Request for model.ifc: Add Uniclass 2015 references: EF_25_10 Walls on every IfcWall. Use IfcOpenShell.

First a look at what the model holds.

```python
import ifcopenshell

model = ifcopenshell.open("model.ifc")
print(model.schema)
print("classifications:", [c.Name for c in model.by_type("IfcClassification")])
for ifc_class in ("IfcDoor", "IfcRoof", "IfcStair", "IfcWall", "IfcWindow"):
    print(ifc_class, len(model.by_type(ifc_class)))
```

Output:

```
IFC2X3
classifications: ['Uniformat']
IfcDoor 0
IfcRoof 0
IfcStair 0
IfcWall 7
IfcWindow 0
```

```python
import ifcopenshell
import ifcopenshell.api.classification

model = ifcopenshell.open("model.ifc")

# IFC2X3 requires Source and Edition and has no link from the project to the system.
system = model.create_entity("IfcClassification", Source="NBS", Edition="2015", Name="Uniclass 2015")

codes = {
    "IfcWall": ("EF_25_10", "Walls"),
}
for ifc_class, (code, name) in codes.items():
    products = model.by_type(ifc_class)
    ifcopenshell.api.classification.add_reference(
        model, products=products, classification=system, identification=code, name=name
    )
    print(code, len(products))

model.write("model-out.ifc")
```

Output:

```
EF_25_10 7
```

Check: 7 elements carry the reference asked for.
